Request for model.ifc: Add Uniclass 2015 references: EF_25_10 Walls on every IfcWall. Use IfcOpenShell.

First a look at what the model holds.

```python
import ifcopenshell

model = ifcopenshell.open("model.ifc")
print(model.schema)
print("classifications:", [c.Name for c in model.by_type("IfcClassification")])
for ifc_class in ("IfcDoor", "IfcRoof", "IfcStair", "IfcWall", "IfcWindow"):
    print(ifc_class, len(model.by_type(ifc_class)))
```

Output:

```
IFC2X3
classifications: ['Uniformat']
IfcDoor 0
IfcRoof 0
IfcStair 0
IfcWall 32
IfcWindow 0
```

```python
import ifcopenshell
import ifcopenshell.api.classification

model = ifcopenshell.open("model.ifc")

# IFC2X3 requires Source and Edition and has no link from the project to the system.
system = model.create_entity("IfcClassification", Source="NBS", Edition="2015", Name="Uniclass 2015")

codes = {
    "IfcWall": ("EF_25_10", "Walls"),
}
for ifc_class, (code, name) in codes.items():
    products = model.by_type(ifc_class)
    ifcopenshell.api.classification.add_reference(
        model, products=products, classification=system, identification=code, name=name
    )
    print(code, len(products))

model.write("model_v2.ifc")
```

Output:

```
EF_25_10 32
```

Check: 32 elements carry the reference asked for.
